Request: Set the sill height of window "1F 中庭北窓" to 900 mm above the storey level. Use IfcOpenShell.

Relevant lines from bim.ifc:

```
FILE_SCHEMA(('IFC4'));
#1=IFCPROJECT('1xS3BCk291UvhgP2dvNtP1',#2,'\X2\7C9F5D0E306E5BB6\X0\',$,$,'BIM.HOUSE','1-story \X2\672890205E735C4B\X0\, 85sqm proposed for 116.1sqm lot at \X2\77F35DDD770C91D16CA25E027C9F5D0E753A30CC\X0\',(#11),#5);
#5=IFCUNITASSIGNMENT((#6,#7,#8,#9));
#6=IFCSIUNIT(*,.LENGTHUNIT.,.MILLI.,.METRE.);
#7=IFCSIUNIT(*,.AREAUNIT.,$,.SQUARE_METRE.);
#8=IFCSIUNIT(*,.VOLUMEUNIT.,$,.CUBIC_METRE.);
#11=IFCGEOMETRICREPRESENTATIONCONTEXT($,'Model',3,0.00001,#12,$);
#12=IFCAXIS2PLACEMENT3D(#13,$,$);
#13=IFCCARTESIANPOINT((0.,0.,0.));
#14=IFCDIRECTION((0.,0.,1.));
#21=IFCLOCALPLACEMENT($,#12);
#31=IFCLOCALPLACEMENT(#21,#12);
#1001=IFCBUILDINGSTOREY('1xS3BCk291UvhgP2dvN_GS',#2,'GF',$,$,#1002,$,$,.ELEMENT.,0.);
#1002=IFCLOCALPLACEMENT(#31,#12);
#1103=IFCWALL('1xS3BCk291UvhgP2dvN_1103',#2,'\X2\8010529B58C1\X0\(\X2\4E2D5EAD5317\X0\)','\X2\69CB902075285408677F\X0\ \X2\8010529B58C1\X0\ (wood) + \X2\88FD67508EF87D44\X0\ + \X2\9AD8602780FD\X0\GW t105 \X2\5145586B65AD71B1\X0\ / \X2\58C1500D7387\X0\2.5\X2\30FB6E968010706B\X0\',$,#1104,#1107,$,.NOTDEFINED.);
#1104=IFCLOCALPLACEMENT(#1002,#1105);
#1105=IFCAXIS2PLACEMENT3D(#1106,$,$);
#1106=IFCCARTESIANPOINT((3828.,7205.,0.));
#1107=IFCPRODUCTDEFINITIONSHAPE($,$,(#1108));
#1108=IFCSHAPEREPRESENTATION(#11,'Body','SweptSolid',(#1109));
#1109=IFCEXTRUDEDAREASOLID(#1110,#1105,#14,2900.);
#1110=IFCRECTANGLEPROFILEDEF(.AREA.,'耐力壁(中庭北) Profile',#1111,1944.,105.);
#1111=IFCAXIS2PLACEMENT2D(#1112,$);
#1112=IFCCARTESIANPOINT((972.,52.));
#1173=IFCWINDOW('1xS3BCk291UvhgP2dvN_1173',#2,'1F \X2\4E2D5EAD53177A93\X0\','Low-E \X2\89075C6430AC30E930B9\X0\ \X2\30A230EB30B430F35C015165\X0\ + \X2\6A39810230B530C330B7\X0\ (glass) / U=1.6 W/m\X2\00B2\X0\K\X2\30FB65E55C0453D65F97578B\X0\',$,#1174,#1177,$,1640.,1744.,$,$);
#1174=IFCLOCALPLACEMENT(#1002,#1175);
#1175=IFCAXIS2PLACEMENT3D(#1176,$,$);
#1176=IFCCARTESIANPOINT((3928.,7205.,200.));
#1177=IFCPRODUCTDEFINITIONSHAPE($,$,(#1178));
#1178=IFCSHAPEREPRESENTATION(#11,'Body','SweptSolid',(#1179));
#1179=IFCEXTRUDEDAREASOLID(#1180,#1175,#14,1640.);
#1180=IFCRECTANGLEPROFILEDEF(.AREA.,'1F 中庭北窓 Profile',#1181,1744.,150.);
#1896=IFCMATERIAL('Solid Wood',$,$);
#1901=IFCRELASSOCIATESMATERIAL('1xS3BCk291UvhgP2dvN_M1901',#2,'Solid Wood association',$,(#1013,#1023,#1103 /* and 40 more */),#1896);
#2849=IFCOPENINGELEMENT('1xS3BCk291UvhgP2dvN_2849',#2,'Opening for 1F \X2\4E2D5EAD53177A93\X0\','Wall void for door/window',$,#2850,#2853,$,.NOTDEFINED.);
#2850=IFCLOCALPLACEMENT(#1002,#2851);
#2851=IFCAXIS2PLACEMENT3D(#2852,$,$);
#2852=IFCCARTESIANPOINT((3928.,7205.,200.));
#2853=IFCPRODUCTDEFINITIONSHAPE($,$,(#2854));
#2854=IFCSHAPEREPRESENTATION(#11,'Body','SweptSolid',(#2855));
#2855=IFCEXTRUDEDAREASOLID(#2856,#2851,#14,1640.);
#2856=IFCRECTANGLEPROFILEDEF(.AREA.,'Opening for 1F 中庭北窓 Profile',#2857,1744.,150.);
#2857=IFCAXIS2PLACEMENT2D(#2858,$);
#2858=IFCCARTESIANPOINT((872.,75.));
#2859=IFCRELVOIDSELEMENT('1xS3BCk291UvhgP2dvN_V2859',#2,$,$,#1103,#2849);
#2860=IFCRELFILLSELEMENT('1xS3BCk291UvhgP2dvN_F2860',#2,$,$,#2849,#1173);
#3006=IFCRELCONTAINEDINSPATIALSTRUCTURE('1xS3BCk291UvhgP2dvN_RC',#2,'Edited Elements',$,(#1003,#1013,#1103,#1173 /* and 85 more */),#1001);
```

```python
import numpy as np
import ifcopenshell
import ifcopenshell.api.geometry
import ifcopenshell.geom
import ifcopenshell.util.element
import ifcopenshell.util.placement
import ifcopenshell.util.shape
import ifcopenshell.util.unit

model = ifcopenshell.open("bim.ifc")
unit_scale = ifcopenshell.util.unit.calculate_unit_scale(model)

window = model.by_guid("1xS3BCk291UvhgP2dvN_1173")
opening = window.FillsVoids[0].RelatingOpeningElement
storey = ifcopenshell.util.element.get_container(window, ifc_class="IfcBuildingStorey")
level = ifcopenshell.util.placement.get_local_placement(storey.ObjectPlacement)[2, 3]

# The opening's origin need not be at the sill, so measure its lowest point.
shape = ifcopenshell.geom.create_shape(ifcopenshell.geom.settings(), opening)
bottom = ifcopenshell.util.shape.get_shape_bottom_elevation(shape, shape.geometry) / unit_scale
dz = level + 0.9 / unit_scale - bottom

shift = np.array([0.0, 0.0, dz])
# The window is not placed relative to its opening, so move both.
for product in (opening, window):
    matrix = ifcopenshell.util.placement.get_local_placement(product.ObjectPlacement)
    matrix[:3, 3] += shift
    ifcopenshell.api.geometry.edit_object_placement(model, product=product, matrix=matrix, is_si=False)

print(f"moved by {dz * unit_scale:+.3f} m")

model.write("bim_v2.ifc")
```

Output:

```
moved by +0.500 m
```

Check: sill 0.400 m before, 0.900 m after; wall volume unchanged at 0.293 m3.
